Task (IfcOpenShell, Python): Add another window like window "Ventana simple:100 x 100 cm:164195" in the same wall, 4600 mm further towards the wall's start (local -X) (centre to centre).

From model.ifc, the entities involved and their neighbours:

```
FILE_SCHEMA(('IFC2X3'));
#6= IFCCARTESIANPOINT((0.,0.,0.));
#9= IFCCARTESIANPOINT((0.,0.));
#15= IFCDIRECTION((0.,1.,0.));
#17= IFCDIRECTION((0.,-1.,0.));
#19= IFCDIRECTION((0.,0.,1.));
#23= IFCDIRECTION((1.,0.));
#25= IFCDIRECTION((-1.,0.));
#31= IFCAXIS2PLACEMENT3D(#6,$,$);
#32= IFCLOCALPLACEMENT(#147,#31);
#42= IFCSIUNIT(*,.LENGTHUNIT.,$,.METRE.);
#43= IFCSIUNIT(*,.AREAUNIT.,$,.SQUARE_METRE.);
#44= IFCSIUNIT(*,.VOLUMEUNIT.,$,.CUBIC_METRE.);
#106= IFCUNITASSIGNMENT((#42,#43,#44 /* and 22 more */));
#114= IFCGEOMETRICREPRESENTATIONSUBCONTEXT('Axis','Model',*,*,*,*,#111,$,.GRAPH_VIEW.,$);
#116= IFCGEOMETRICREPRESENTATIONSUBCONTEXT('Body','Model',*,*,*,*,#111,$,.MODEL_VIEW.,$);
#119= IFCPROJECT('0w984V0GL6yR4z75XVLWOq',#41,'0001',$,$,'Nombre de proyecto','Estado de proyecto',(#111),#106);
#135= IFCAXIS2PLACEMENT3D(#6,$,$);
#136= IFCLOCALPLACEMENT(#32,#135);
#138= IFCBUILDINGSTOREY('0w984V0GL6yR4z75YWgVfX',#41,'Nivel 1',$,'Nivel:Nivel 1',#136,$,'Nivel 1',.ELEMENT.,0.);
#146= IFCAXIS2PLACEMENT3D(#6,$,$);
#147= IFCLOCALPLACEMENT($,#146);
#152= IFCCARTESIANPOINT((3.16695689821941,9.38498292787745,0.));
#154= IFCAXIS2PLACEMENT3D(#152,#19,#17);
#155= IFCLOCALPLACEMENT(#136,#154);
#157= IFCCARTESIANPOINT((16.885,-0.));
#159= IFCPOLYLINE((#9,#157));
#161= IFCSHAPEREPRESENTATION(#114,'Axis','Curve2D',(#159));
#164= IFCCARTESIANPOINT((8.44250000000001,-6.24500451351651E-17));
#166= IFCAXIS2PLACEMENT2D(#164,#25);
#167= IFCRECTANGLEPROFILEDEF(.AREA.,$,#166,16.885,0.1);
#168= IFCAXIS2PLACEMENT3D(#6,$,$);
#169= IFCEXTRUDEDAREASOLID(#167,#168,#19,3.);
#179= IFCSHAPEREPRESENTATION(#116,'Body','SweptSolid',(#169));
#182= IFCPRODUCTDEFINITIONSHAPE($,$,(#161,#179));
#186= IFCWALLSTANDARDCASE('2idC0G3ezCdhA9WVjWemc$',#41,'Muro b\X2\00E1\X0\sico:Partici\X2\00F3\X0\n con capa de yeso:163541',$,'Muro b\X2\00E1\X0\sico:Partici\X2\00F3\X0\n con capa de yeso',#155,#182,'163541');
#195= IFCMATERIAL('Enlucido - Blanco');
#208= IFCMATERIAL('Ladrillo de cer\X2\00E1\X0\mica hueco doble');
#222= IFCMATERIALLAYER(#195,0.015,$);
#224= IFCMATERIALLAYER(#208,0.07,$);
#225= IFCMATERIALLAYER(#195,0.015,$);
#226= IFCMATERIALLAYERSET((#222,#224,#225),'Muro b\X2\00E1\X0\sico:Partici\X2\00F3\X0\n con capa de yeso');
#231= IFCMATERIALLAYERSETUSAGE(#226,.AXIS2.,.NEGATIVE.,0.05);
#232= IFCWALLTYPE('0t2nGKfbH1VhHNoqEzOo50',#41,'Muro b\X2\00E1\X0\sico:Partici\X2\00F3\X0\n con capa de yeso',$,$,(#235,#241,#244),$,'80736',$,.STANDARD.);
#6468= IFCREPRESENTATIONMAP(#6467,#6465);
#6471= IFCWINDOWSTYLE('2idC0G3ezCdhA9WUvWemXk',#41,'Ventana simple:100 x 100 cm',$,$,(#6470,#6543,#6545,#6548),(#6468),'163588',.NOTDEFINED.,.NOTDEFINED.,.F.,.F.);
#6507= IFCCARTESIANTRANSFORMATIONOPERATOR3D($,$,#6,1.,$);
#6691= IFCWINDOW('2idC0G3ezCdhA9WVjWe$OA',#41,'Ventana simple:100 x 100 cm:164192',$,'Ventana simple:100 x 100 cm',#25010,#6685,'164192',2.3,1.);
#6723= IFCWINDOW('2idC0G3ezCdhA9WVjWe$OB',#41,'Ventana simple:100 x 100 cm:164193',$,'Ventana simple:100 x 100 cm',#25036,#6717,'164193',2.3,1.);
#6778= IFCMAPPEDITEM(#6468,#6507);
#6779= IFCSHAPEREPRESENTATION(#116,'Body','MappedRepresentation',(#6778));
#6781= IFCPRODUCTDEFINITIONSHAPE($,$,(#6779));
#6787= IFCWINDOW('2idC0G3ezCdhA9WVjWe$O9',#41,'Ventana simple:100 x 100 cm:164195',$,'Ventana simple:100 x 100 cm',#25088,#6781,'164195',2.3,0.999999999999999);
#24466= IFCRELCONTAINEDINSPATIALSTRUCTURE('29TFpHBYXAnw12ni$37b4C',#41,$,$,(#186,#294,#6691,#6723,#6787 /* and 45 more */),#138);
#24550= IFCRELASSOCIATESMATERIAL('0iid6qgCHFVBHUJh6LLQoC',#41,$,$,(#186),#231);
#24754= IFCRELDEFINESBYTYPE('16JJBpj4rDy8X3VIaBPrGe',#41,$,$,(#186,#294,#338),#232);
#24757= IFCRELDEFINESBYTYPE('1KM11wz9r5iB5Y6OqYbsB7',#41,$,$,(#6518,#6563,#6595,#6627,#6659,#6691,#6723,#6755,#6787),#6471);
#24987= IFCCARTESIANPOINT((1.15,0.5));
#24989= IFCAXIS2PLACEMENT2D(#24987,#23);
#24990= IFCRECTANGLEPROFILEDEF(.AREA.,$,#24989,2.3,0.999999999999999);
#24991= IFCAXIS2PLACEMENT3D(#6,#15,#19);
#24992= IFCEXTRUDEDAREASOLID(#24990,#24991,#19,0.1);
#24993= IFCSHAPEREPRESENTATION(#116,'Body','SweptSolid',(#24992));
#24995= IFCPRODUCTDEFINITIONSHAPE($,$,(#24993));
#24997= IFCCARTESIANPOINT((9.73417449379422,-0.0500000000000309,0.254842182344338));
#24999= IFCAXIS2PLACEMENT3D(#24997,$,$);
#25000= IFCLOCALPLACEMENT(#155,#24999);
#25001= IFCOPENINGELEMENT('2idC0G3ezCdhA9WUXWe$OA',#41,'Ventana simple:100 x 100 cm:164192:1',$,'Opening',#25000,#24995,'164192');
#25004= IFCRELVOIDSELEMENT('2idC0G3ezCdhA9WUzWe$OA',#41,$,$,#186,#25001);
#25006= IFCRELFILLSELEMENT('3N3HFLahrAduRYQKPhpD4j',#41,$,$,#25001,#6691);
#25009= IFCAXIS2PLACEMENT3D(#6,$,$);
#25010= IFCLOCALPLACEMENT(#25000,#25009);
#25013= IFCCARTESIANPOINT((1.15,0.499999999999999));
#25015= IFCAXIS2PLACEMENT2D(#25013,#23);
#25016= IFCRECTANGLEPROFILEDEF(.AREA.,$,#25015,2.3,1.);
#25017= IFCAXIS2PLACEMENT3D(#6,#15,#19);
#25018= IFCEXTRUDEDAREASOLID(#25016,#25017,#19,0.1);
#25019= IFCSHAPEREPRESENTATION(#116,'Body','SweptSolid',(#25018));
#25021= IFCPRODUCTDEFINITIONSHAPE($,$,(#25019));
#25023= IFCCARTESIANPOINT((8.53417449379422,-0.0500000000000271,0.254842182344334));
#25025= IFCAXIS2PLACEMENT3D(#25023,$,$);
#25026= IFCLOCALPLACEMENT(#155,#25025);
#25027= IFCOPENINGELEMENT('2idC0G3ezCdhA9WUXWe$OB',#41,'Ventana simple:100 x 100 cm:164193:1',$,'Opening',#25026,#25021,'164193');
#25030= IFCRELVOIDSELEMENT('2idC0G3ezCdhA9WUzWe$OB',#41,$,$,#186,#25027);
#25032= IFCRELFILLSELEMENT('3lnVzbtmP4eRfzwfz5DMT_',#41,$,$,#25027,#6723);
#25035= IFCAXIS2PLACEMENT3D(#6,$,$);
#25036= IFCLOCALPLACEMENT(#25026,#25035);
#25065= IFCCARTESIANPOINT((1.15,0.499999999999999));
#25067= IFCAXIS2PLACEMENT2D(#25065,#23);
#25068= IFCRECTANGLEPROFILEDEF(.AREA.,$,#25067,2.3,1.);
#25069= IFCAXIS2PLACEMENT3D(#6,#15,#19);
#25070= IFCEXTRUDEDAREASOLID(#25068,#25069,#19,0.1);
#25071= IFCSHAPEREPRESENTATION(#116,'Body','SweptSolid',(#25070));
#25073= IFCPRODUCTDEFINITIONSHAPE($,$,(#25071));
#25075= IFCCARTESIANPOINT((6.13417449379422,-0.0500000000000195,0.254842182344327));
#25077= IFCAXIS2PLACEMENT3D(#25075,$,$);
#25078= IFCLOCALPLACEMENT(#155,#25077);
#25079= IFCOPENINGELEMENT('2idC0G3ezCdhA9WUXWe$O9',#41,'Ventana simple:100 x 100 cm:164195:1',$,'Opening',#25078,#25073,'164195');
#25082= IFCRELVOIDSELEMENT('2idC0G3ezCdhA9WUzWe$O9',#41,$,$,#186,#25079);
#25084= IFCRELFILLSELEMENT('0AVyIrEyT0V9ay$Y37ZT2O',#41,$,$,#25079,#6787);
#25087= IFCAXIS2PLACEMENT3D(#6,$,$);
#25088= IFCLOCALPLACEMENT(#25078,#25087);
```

```python
import ifcopenshell
import ifcopenshell.api.feature
import ifcopenshell.api.geometry
import ifcopenshell.api.root
import ifcopenshell.geom
import ifcopenshell.util.element
import ifcopenshell.util.placement
import ifcopenshell.util.shape
import ifcopenshell.util.unit

model = ifcopenshell.open("model.ifc")
unit_scale = ifcopenshell.util.unit.calculate_unit_scale(model)
settings = ifcopenshell.geom.settings()


def volume(element):
    """Net volume in cubic metres, openings subtracted."""
    shape = ifcopenshell.geom.create_shape(settings, element)
    return ifcopenshell.util.shape.get_volume(shape.geometry)


def reuse_history(source, copy):
    """copy_class also copies each property set's owner history, people and application; keep the originals."""
    for rel in copy.IsDefinedBy:
        if rel.is_a("IfcRelDefinesByProperties") and (history := rel.RelatingPropertyDefinition.OwnerHistory):
            rel.RelatingPropertyDefinition.OwnerHistory = source.OwnerHistory
            ifcopenshell.util.element.remove_deep2(model, history)


window = model.by_guid("2idC0G3ezCdhA9WVjWe$O9")
opening = window.FillsVoids[0].RelatingOpeningElement
wall = opening.VoidsElements[0].RelatingBuildingElement
before = volume(wall)
shift = ifcopenshell.util.placement.get_local_placement(wall.ObjectPlacement)[:3, 0] * -4.6 / unit_scale

# copy_class copies the void relationship, type, container and properties, but no geometry.
new_opening = ifcopenshell.api.root.copy_class(model, product=opening)
new_opening.Representation = ifcopenshell.util.element.copy_deep(
    model, opening.Representation, exclude=["IfcGeometricRepresentationContext", "IfcRepresentationMap"]
)
new_opening.Name = "Ventana simple:100 x 100 cm"
new_opening.Tag = None
new_window = ifcopenshell.api.root.copy_class(model, product=window)
new_window.Representation = ifcopenshell.util.element.copy_deep(
    model, window.Representation, exclude=["IfcGeometricRepresentationContext", "IfcRepresentationMap"]
)
new_window.Name = "Ventana simple:100 x 100 cm"
new_window.Tag = None
reuse_history(window, new_window)
fills = ifcopenshell.api.feature.add_filling(model, opening=new_opening, element=new_window)
fills.OwnerHistory = new_window.OwnerHistory  # required in IFC2X3

for old, new in ((opening, new_opening), (window, new_window)):
    matrix = ifcopenshell.util.placement.get_local_placement(old.ObjectPlacement)
    matrix[:3, 3] += shift
    ifcopenshell.api.geometry.edit_object_placement(model, product=new, matrix=matrix, is_si=False)

after = volume(wall)

print(f"wall volume {before:.3f} -> {after:.3f} m3")

model.write("model-out.ifc")
```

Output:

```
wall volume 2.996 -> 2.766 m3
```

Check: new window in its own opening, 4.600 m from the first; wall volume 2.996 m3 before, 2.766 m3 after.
